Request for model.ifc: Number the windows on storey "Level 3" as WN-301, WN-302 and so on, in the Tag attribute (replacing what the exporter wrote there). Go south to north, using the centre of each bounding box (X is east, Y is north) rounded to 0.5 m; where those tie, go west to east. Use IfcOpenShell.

First a look at what the model holds.

```python
import ifcopenshell
import ifcopenshell.util.element
import ifcopenshell.util.placement

model = ifcopenshell.open("model.ifc")
print(model.schema)
storey = next(s for s in model.by_type("IfcBuildingStorey") if s.Name == "Level 3")
windows = [e for e in ifcopenshell.util.element.get_decomposition(storey) if e.is_a("IfcWindow")]
for e in sorted(windows, key=lambda e: e.id()):
    origin = ifcopenshell.util.placement.get_local_placement(e.ObjectPlacement)[:3, 3]
    print(e.id(), e.Tag, e.Name, origin.round(2) + 0.0, sep=" | ")
```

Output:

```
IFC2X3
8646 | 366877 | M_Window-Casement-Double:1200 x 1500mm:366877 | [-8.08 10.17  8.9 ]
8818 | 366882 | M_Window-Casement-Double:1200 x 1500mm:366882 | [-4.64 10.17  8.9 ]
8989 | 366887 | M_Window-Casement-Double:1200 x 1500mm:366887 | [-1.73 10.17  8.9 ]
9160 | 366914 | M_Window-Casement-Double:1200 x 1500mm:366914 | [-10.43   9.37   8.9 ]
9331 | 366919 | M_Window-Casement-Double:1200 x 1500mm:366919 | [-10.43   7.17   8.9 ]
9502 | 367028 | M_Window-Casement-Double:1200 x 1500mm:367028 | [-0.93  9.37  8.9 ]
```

```python
import ifcopenshell
import ifcopenshell.geom
import ifcopenshell.util.element
import ifcopenshell.util.shape

model = ifcopenshell.open("model.ifc")
settings = ifcopenshell.geom.settings()
settings.set("use-world-coords", True)


def centre(element):
    shape = ifcopenshell.geom.create_shape(settings, element)
    return ifcopenshell.util.shape.get_bbox_centroid(shape.geometry)


storey = next(s for s in model.by_type("IfcBuildingStorey") if s.Name == "Level 3")
windows = [e for e in ifcopenshell.util.element.get_decomposition(storey) if e.is_a("IfcWindow")]

# Insertion points can sit at a corner or the storey origin, so sort by the geometry (in metres).
centres = {e: centre(e) for e in windows}
windows.sort(key=lambda e: (round(centres[e][1] / 0.5), centres[e][0]))

for i, e in enumerate(windows, start=1):
    number = f"WN-3{i:02d}"
    e.Tag = number
    print(e.id(), number)

model.write("model_rev.ifc")
```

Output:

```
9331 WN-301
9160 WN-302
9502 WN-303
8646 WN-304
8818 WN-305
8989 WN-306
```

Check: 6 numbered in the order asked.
